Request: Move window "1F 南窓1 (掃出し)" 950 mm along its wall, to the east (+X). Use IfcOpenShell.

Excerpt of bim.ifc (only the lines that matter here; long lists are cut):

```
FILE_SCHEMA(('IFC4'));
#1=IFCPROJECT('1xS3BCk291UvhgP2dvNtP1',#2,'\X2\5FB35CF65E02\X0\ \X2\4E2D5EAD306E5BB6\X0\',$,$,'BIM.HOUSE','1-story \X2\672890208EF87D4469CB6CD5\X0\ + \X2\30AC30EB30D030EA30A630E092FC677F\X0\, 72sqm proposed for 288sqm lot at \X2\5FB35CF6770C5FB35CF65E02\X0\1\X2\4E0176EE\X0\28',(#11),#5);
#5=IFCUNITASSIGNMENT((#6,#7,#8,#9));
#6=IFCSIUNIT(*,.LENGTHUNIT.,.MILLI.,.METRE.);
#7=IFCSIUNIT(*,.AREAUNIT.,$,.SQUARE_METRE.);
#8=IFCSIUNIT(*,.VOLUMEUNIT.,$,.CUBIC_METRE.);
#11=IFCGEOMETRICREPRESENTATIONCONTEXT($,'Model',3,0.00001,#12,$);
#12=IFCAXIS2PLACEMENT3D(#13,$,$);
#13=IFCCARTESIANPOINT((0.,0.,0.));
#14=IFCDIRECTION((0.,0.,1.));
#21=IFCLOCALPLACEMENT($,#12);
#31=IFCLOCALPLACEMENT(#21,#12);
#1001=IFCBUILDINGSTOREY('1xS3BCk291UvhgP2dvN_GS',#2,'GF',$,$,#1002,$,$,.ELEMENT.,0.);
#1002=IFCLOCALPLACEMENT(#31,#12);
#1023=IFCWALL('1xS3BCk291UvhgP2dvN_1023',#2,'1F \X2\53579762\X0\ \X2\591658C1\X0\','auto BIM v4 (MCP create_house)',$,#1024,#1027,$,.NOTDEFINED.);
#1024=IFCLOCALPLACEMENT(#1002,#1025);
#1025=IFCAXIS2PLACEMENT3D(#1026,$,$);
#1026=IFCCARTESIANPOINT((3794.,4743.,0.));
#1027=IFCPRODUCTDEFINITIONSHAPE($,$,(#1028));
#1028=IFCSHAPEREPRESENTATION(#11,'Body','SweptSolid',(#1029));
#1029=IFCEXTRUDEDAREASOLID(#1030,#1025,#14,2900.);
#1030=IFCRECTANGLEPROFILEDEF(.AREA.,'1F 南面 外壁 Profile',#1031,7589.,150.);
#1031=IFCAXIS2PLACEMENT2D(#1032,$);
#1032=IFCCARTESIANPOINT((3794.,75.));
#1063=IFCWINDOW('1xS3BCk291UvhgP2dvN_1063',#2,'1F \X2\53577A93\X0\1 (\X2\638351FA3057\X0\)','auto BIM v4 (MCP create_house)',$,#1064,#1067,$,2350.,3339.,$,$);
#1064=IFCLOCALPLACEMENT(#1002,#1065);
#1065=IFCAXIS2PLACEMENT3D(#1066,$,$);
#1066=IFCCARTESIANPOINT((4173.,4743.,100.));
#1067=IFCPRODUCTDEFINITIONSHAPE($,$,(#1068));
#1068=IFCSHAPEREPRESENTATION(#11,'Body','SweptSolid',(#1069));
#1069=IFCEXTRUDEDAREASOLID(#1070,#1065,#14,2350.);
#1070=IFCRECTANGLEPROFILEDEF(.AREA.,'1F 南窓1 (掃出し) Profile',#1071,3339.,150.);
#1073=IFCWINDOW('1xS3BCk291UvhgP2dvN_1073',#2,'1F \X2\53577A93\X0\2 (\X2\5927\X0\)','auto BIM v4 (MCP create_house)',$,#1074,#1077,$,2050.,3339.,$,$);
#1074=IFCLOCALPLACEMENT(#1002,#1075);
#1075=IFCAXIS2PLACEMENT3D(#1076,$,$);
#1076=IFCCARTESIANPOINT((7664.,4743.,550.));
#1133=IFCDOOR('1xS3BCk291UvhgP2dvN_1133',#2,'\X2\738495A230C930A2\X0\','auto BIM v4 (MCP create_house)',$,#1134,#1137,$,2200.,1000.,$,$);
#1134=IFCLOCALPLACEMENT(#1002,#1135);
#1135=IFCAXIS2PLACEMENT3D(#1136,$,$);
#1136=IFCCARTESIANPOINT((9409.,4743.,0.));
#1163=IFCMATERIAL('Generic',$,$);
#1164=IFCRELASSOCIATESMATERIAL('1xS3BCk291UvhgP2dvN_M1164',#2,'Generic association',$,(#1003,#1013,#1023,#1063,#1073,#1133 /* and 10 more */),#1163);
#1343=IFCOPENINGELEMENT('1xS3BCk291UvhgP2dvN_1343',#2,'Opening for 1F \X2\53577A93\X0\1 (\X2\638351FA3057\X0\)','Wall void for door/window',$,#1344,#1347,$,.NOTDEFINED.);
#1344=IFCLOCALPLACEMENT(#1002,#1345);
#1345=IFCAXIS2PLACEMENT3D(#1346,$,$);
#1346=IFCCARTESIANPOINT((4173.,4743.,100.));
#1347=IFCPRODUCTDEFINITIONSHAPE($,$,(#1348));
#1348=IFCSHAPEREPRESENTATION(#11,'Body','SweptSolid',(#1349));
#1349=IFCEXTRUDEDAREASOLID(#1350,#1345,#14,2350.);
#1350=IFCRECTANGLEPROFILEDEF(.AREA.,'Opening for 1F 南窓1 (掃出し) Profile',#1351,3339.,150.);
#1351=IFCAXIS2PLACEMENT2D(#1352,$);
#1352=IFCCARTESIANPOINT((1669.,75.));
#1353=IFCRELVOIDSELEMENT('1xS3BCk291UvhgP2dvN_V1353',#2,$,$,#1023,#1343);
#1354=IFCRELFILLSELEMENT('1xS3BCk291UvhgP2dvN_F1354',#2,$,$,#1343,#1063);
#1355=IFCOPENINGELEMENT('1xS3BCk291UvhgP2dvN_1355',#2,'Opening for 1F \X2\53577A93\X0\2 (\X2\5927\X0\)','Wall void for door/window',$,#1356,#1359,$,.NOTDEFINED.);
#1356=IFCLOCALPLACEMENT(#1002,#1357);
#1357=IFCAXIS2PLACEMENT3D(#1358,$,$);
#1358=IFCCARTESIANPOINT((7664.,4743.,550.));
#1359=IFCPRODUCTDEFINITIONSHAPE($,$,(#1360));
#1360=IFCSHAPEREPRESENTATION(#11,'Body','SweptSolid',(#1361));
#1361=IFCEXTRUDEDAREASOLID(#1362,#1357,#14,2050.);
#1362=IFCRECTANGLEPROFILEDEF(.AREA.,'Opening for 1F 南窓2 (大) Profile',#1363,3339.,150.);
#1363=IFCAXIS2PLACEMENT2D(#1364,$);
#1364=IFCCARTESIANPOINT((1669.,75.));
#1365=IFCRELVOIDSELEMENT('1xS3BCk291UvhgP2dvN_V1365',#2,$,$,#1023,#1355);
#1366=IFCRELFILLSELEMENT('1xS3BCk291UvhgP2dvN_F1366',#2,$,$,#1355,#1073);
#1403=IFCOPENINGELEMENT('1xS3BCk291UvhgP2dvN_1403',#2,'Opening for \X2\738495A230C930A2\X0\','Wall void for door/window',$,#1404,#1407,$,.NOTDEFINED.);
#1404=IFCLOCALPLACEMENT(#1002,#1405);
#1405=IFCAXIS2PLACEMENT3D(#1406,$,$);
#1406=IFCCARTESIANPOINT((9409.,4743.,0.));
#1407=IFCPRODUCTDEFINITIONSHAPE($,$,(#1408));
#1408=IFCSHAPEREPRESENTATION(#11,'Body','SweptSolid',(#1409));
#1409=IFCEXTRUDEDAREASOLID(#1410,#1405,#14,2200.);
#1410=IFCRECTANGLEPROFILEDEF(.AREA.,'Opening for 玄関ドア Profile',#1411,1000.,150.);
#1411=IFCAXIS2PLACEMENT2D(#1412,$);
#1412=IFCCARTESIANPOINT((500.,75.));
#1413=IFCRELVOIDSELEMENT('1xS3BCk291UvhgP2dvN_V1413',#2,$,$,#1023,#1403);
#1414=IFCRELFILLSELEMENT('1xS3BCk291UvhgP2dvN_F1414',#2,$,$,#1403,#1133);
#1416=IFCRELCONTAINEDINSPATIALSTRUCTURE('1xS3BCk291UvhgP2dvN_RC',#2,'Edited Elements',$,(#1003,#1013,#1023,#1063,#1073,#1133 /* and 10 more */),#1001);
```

```python
import ifcopenshell
import ifcopenshell.api.geometry
import ifcopenshell.util.placement

model = ifcopenshell.open("bim.ifc")

window = model.by_guid("1xS3BCk291UvhgP2dvN_1063")
opening = window.FillsVoids[0].RelatingOpeningElement
wall = opening.VoidsElements[0].RelatingBuildingElement

wall_matrix = ifcopenshell.util.placement.get_local_placement(wall.ObjectPlacement)
shift = wall_matrix[:3, 0] * 950.0
before = ifcopenshell.util.placement.get_local_placement(window.ObjectPlacement)[:3, 3].copy()

# The window is not placed relative to its opening, so move both.
for product in (opening, window):
    matrix = ifcopenshell.util.placement.get_local_placement(product.ObjectPlacement)
    matrix[:3, 3] += shift
    ifcopenshell.api.geometry.edit_object_placement(model, product=product, matrix=matrix, is_si=False)

after = ifcopenshell.util.placement.get_local_placement(window.ObjectPlacement)[:3, 3]
print("window moved by", (after - before).round(3) + 0.0)

model.write("bim_edited.ifc")
```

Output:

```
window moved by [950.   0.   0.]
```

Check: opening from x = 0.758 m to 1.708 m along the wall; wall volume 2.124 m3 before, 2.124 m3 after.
